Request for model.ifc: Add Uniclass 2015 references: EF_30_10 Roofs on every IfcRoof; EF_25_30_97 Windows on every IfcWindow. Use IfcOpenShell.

First a look at what the model holds.

```python
import ifcopenshell

model = ifcopenshell.open("model.ifc")
print(model.schema)
print("classifications:", [c.Name for c in model.by_type("IfcClassification")])
for ifc_class in ("IfcDoor", "IfcRoof", "IfcStair", "IfcWall", "IfcWindow"):
    print(ifc_class, len(model.by_type(ifc_class)))
```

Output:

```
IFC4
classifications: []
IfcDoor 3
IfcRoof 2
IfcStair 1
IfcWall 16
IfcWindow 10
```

```python
import ifcopenshell
import ifcopenshell.api.classification

model = ifcopenshell.open("model.ifc")

system = ifcopenshell.api.classification.add_classification(model, classification="Uniclass 2015")

codes = {
    "IfcRoof": ("EF_30_10", "Roofs"),
    "IfcWindow": ("EF_25_30_97", "Windows"),
}
for ifc_class, (code, name) in codes.items():
    products = model.by_type(ifc_class)
    ifcopenshell.api.classification.add_reference(
        model, products=products, classification=system, identification=code, name=name
    )
    print(code, len(products))

model.write("model_edited.ifc")
```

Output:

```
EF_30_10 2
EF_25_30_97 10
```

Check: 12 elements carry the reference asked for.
